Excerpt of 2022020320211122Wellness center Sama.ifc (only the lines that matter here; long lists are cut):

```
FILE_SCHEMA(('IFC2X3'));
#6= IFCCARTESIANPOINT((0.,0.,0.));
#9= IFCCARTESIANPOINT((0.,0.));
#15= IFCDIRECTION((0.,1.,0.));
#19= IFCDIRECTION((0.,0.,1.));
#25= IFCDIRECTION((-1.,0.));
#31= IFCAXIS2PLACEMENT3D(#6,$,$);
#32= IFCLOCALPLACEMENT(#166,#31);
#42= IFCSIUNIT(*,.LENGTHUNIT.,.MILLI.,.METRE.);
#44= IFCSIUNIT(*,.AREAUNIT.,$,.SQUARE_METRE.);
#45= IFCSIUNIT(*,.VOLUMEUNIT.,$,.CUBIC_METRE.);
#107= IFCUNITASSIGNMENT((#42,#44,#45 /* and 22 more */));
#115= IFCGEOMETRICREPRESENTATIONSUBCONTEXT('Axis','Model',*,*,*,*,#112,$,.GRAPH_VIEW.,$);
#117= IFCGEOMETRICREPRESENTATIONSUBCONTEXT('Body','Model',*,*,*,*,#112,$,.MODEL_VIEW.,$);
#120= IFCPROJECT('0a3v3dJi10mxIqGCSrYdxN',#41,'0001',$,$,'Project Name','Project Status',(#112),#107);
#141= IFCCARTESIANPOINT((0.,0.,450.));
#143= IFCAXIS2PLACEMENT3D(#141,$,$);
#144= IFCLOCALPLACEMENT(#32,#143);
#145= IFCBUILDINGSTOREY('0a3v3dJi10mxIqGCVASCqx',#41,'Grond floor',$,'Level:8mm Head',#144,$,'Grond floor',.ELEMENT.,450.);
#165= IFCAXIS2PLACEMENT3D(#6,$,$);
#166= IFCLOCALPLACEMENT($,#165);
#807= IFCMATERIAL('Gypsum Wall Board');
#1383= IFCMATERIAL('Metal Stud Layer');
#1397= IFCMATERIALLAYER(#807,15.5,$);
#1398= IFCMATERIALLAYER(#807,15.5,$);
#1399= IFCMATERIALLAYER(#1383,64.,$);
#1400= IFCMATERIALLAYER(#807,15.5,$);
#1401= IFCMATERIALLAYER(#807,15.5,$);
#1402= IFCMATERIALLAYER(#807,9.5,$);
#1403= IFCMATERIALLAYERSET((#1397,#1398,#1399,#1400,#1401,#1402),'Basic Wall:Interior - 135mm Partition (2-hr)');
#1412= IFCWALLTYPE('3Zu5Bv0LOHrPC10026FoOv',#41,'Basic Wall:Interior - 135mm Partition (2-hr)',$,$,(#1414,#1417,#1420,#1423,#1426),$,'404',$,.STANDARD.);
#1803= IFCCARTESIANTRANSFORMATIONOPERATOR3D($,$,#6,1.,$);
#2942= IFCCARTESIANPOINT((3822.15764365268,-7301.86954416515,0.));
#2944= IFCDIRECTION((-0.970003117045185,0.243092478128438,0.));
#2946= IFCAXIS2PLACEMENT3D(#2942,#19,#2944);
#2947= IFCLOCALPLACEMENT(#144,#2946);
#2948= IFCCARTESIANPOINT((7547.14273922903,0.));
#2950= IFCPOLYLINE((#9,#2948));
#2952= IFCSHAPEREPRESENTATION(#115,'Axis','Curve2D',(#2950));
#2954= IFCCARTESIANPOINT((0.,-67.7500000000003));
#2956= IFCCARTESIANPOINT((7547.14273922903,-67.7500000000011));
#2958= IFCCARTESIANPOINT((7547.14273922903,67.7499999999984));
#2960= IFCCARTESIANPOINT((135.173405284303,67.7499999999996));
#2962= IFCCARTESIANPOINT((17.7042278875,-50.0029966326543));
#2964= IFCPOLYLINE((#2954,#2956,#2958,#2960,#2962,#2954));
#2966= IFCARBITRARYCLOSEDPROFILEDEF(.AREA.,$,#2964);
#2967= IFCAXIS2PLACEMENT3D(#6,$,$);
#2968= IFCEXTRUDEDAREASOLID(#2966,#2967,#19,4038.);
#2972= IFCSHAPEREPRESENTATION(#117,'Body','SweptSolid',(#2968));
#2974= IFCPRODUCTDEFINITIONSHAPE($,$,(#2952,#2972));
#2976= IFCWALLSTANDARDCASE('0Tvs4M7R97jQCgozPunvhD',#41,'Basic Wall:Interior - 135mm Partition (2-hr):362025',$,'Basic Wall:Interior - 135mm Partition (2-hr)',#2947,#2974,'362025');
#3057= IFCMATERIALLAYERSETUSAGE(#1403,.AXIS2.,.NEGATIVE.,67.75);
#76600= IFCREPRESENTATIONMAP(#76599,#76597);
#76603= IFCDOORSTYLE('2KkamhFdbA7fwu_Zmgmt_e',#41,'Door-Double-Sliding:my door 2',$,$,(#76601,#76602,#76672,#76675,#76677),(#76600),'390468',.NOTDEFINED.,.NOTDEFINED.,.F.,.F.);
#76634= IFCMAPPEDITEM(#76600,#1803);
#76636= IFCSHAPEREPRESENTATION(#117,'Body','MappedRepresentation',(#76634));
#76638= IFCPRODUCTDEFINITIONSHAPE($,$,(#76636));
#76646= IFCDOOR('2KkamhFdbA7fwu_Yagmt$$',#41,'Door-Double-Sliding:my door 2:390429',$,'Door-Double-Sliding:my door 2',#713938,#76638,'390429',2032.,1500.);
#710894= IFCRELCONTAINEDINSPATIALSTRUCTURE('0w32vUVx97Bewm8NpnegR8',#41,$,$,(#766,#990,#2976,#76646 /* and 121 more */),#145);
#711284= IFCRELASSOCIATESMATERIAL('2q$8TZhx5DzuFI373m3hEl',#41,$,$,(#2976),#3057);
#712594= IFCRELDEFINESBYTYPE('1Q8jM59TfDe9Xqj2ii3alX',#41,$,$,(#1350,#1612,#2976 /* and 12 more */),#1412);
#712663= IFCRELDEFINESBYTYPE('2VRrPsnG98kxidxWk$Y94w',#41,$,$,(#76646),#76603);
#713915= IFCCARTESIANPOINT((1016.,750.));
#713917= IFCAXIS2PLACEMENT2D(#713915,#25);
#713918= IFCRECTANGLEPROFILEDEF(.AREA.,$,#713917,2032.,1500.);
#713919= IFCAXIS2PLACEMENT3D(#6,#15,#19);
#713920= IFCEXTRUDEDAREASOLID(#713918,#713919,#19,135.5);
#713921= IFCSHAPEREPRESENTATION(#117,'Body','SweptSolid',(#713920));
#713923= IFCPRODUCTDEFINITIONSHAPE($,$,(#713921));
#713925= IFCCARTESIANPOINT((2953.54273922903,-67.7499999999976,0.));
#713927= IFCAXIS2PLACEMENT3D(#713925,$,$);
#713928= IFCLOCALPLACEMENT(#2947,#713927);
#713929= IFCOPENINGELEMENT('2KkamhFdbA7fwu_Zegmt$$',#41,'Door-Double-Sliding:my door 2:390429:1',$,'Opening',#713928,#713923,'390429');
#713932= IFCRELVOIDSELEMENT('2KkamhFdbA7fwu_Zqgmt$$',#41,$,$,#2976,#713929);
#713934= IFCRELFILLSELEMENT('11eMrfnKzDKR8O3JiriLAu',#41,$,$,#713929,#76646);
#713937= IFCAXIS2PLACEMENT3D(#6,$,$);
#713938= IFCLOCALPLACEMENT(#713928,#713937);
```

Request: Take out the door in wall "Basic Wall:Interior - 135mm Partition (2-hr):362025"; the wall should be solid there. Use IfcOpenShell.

```python
import ifcopenshell
import ifcopenshell.api.feature
import ifcopenshell.api.root
import ifcopenshell.geom
import ifcopenshell.util.shape

model = ifcopenshell.open("2022020320211122Wellness center Sama.ifc")
settings = ifcopenshell.geom.settings()


def volume(element):
    """Net volume in cubic metres, openings subtracted."""
    shape = ifcopenshell.geom.create_shape(settings, element)
    return ifcopenshell.util.shape.get_volume(shape.geometry)


door = model.by_id(76646)
opening = door.FillsVoids[0].RelatingOpeningElement
wall = opening.VoidsElements[0].RelatingBuildingElement
before = volume(wall)

ifcopenshell.api.root.remove_product(model, product=door)
ifcopenshell.api.feature.remove_feature(model, feature=opening)

after = volume(wall)

print(f"wall volume {before:.3f} -> {after:.3f} m3")

model.write("2022020320211122Wellness center Sama_rev.ifc")
```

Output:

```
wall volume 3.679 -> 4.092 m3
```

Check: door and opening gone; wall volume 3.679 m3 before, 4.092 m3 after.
